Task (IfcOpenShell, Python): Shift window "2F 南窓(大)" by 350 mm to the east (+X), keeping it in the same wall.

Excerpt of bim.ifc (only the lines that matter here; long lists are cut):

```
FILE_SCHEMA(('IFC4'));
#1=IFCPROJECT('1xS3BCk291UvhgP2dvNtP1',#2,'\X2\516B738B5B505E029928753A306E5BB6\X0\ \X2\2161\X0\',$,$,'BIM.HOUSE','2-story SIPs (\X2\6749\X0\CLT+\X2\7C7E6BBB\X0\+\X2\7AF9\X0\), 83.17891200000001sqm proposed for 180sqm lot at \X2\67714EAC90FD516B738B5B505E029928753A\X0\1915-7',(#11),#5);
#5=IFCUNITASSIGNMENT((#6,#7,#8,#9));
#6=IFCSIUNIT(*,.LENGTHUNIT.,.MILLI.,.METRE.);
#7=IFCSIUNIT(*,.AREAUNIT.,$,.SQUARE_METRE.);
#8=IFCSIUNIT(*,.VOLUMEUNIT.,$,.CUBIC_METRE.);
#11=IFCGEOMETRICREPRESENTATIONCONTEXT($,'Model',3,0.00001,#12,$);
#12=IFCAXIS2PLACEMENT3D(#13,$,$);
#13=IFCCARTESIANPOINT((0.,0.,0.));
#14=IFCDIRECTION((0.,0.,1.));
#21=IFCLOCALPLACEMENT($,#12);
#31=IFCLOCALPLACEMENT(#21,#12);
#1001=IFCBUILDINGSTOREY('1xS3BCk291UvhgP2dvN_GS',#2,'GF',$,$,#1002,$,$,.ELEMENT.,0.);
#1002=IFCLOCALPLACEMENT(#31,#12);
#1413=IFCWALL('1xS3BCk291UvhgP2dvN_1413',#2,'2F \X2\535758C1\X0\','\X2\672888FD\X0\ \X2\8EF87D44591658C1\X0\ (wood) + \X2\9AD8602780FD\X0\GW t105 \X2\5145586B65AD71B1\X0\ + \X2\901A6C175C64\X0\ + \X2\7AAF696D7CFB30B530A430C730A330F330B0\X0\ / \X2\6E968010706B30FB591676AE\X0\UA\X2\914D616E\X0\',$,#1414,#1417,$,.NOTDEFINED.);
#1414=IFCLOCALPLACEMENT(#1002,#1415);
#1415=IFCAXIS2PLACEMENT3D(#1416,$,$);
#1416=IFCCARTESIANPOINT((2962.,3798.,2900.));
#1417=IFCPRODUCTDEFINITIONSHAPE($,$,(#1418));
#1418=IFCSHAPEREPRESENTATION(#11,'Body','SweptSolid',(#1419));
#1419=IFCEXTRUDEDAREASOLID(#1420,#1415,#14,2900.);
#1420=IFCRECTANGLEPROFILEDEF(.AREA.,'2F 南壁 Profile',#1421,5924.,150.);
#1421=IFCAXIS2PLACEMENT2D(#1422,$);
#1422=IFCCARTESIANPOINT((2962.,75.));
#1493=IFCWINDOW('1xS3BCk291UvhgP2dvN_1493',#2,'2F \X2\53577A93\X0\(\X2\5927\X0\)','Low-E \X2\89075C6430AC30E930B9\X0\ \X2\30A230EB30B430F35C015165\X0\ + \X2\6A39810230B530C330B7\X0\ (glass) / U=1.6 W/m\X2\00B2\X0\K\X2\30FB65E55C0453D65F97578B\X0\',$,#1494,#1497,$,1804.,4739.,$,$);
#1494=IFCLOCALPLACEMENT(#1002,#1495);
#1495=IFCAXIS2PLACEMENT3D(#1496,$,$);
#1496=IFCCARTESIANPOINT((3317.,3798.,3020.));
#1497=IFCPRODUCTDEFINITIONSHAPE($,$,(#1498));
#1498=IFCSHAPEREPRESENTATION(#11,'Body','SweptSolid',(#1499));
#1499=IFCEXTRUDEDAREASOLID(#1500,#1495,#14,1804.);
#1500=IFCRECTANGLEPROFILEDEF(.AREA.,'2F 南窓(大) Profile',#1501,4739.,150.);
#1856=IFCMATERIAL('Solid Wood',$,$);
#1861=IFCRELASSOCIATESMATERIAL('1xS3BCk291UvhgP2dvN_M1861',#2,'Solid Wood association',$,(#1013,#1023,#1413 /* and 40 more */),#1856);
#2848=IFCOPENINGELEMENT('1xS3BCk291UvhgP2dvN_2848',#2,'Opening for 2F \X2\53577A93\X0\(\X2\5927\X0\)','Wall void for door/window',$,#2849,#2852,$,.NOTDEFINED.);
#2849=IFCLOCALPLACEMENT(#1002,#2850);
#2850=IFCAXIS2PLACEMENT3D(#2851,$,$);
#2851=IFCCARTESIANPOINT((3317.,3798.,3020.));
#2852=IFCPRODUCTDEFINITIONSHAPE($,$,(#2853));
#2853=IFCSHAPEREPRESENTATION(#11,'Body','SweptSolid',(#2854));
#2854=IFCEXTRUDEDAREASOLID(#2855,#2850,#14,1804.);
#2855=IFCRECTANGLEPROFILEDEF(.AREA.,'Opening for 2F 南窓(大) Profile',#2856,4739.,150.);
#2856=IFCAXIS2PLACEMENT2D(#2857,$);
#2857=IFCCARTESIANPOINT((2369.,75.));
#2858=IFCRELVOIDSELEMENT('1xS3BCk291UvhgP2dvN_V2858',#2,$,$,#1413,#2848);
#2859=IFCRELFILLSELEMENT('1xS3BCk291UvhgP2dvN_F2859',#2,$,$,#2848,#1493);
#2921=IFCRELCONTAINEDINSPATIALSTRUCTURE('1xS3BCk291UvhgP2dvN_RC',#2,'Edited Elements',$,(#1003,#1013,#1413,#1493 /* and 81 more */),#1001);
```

```python
import ifcopenshell
import ifcopenshell.api.geometry
import ifcopenshell.util.placement
import ifcopenshell.util.unit

model = ifcopenshell.open("bim.ifc")
unit_scale = ifcopenshell.util.unit.calculate_unit_scale(model)

window = model.by_guid("1xS3BCk291UvhgP2dvN_1493")
opening = window.FillsVoids[0].RelatingOpeningElement
wall = opening.VoidsElements[0].RelatingBuildingElement

wall_matrix = ifcopenshell.util.placement.get_local_placement(wall.ObjectPlacement)
shift = wall_matrix[:3, 0] * 0.35 / unit_scale
before = ifcopenshell.util.placement.get_local_placement(window.ObjectPlacement)[:3, 3].copy()

# The window is not placed relative to its opening, so move both.
for product in (opening, window):
    matrix = ifcopenshell.util.placement.get_local_placement(product.ObjectPlacement)
    matrix[:3, 3] += shift
    ifcopenshell.api.geometry.edit_object_placement(model, product=product, matrix=matrix, is_si=False)

after = ifcopenshell.util.placement.get_local_placement(window.ObjectPlacement)[:3, 3]
print("window moved by", (after - before).round(3) + 0.0)

model.write("bim-out.ifc")
```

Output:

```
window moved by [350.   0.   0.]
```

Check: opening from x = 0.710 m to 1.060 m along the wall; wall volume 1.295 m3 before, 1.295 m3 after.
